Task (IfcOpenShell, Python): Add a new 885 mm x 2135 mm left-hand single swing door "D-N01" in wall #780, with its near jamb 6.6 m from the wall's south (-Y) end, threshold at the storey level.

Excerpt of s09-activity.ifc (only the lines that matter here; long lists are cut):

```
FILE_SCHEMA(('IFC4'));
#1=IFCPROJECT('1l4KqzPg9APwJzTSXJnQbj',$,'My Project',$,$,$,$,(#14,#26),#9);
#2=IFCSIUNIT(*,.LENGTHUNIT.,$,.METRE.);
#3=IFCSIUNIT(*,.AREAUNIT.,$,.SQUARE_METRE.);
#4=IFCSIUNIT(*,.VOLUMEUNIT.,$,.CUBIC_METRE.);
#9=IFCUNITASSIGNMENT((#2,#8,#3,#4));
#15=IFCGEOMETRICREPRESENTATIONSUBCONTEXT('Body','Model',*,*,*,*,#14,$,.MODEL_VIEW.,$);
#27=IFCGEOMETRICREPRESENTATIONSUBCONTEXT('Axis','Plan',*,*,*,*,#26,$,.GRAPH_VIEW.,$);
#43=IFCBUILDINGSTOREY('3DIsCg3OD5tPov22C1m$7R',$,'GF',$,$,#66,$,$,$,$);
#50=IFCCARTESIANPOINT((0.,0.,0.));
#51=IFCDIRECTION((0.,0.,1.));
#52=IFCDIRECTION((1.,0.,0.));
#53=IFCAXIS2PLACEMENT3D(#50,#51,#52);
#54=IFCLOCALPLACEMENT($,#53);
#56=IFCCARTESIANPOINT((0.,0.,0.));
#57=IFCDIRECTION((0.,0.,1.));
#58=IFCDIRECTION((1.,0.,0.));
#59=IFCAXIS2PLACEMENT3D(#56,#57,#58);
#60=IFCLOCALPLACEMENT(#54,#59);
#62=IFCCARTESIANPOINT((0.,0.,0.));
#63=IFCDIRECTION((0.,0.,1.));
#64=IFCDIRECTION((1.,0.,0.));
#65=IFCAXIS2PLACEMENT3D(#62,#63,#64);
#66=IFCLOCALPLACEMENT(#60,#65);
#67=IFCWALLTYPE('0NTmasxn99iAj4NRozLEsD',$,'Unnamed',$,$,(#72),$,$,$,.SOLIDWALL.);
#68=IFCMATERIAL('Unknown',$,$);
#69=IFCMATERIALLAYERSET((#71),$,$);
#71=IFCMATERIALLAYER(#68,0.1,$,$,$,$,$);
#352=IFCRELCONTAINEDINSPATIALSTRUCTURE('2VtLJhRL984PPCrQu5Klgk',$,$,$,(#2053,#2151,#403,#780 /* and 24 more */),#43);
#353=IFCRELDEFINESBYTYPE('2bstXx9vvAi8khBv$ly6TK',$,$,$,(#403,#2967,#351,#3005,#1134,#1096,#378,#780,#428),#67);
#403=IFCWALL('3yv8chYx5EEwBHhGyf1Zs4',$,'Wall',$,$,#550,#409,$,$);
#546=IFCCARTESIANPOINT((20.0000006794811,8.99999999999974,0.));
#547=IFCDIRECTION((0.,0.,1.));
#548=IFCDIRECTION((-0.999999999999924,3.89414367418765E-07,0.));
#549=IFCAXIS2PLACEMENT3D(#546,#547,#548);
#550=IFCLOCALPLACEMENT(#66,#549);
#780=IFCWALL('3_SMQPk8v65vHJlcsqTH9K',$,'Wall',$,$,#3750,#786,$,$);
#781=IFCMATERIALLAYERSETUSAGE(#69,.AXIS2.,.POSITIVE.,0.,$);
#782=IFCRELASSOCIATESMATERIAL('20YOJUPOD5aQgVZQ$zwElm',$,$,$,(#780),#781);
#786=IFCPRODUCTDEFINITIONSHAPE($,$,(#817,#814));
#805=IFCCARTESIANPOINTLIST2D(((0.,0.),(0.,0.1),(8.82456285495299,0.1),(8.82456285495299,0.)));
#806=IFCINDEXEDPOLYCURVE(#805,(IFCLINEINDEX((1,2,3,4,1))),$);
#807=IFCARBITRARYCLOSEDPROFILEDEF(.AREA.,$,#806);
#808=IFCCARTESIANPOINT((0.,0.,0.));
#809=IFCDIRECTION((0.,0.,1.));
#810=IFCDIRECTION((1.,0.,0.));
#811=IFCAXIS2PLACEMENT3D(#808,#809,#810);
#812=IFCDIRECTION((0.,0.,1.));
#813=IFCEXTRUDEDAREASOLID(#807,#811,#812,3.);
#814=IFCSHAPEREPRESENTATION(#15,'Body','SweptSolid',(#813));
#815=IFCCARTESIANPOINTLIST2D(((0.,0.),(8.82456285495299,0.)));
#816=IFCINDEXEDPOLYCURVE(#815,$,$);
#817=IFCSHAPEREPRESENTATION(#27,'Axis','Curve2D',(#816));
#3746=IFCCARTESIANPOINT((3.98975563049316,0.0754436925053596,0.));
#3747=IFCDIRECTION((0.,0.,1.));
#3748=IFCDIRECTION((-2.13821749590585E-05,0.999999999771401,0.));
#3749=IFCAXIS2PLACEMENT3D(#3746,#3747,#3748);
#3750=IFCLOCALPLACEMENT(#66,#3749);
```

```python
import numpy as np
import ifcopenshell
import ifcopenshell.api.feature
import ifcopenshell.api.geometry
import ifcopenshell.api.root
import ifcopenshell.api.spatial
import ifcopenshell.geom
import ifcopenshell.util.element
import ifcopenshell.util.placement
import ifcopenshell.util.representation
import ifcopenshell.util.shape
import ifcopenshell.util.unit

model = ifcopenshell.open("s09-activity.ifc")
unit_scale = ifcopenshell.util.unit.calculate_unit_scale(model)
settings = ifcopenshell.geom.settings()


def volume(element):
    """Net volume in cubic metres, openings subtracted."""
    shape = ifcopenshell.geom.create_shape(settings, element)
    return ifcopenshell.util.shape.get_volume(shape.geometry)


wall = model.by_guid("3_SMQPk8v65vHJlcsqTH9K")
storey = ifcopenshell.util.element.get_container(wall, ifc_class="IfcBuildingStorey")
context = ifcopenshell.util.representation.get_context(model, "Model", "Body", "MODEL_VIEW")
before = volume(wall)

width, height, from_end, sill = 0.885, 2.135, 6.6, 0.0  # metres

# The wall runs along its own X axis, and the end named is its -X end.
wall_shape = ifcopenshell.geom.create_shape(settings, wall)
x, y, z = ifcopenshell.util.shape.get_vertices(wall_shape.geometry).T
start = x.min() + from_end
face, thickness = float(y.min()), float(y.max() - y.min())
wall_matrix = ifcopenshell.util.placement.get_local_placement(wall.ObjectPlacement)
level = ifcopenshell.util.placement.get_local_placement(storey.ObjectPlacement)[2, 3]


def in_wall(x, y):
    """Placement at x, y metres in the wall's axes, at sill height."""
    matrix = wall_matrix.copy()
    matrix[:, 3] = wall_matrix @ np.array([x / unit_scale, y / unit_scale, 0.0, 1.0])
    matrix[2, 3] = level + sill / unit_scale
    return matrix


# Opening: a box that overshoots both wall faces by 50 mm.
opening = ifcopenshell.api.root.create_entity(model, ifc_class="IfcOpeningElement", predefined_type="OPENING")
box = ifcopenshell.api.geometry.add_wall_representation(
    model, context=context, length=width, height=height, thickness=thickness + 0.1
)
ifcopenshell.api.geometry.assign_representation(model, product=opening, representation=box)
ifcopenshell.api.geometry.edit_object_placement(model, product=opening, matrix=in_wall(start, face - 0.05), is_si=False)
ifcopenshell.api.feature.add_feature(model, feature=opening, element=wall)

door = ifcopenshell.api.root.create_entity(model, ifc_class="IfcDoor", name="D-N01", predefined_type="DOOR")
door.OverallWidth, door.OverallHeight = width / unit_scale, height / unit_scale
door.OperationType = "SINGLE_SWING_LEFT"
body = ifcopenshell.api.geometry.add_door_representation(
    model,
    context=context,
    overall_width=door.OverallWidth,
    overall_height=door.OverallHeight,
    operation_type="SINGLE_SWING_LEFT",
    lining_properties={"LiningDepth": thickness / unit_scale, "ThresholdDepth": thickness / unit_scale},
)
ifcopenshell.api.geometry.assign_representation(model, product=door, representation=body)
ifcopenshell.api.spatial.assign_container(model, products=[door], relating_structure=storey)
ifcopenshell.api.feature.add_filling(model, opening=opening, element=door)

# The lining spans the wall, so the door starts at the wall face.
ifcopenshell.api.geometry.edit_object_placement(model, product=door, matrix=in_wall(start, face), is_si=False)

after = volume(wall)

print(f"wall volume {before:.3f} -> {after:.3f} m3")

model.write("s09-activity_rev.ifc")
```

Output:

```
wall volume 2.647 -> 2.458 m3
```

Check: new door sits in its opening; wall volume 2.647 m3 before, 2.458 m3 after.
